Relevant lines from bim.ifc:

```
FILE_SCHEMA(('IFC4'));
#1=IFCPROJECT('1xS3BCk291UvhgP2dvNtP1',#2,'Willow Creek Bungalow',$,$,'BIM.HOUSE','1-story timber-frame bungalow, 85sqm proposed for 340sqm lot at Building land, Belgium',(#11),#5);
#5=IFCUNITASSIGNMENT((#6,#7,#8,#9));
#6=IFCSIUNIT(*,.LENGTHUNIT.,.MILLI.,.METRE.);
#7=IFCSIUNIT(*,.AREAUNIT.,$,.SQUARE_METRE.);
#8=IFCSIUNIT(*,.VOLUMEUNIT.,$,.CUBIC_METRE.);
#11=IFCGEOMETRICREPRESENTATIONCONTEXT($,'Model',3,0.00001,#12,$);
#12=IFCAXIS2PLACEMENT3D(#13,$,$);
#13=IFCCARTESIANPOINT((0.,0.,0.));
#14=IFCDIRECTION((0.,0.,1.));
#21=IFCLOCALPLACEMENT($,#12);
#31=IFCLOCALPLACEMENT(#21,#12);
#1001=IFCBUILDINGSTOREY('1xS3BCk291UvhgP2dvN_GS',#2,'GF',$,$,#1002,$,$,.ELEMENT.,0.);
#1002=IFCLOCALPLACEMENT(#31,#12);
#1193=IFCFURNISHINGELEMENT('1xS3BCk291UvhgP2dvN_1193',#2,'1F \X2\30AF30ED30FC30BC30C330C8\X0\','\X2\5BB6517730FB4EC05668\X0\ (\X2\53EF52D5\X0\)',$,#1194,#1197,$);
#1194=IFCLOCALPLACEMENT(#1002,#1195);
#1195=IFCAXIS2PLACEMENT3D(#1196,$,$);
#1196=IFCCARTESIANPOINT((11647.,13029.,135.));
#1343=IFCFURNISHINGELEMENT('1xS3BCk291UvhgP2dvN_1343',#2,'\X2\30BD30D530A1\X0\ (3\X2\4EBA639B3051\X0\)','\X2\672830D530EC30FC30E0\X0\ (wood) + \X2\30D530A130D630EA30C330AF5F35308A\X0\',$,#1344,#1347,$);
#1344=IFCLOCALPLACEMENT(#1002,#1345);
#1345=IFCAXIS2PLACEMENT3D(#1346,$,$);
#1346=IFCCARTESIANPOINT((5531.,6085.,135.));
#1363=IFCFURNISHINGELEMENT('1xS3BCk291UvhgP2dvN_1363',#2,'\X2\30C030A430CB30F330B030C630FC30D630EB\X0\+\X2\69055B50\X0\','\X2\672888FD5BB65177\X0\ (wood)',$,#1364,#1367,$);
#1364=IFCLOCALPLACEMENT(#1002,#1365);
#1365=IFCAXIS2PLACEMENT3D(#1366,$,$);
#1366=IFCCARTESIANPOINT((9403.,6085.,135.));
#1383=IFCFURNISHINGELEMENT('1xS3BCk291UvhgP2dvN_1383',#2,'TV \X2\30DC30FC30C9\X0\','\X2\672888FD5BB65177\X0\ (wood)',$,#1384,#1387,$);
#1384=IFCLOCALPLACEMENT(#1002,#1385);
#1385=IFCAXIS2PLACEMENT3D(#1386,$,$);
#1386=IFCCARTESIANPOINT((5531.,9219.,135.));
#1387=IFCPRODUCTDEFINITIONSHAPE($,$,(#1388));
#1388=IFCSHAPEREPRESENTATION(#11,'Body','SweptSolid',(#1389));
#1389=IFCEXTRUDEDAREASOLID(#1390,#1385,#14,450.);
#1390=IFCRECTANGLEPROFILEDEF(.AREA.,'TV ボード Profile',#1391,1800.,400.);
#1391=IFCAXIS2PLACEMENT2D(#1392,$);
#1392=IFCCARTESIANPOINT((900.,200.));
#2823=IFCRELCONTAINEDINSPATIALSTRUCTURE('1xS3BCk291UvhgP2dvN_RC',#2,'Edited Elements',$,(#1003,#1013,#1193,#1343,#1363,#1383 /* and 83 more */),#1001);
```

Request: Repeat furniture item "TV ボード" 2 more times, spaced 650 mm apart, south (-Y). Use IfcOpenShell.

```python
import numpy as np
import ifcopenshell
import ifcopenshell.api.geometry
import ifcopenshell.api.root
import ifcopenshell.util.element
import ifcopenshell.util.placement
import ifcopenshell.util.unit

model = ifcopenshell.open("bim.ifc")
unit_scale = ifcopenshell.util.unit.calculate_unit_scale(model)


def reuse_history(source, copy):
    """copy_class also copies each property set's owner history, people and application; keep the originals."""
    for rel in copy.IsDefinedBy:
        if rel.is_a("IfcRelDefinesByProperties") and (history := rel.RelatingPropertyDefinition.OwnerHistory):
            rel.RelatingPropertyDefinition.OwnerHistory = source.OwnerHistory
            ifcopenshell.util.element.remove_deep2(model, history)


source = model.by_id(1383)
base = ifcopenshell.util.placement.get_local_placement(source.ObjectPlacement)
step = np.array([0.0, -1.0, 0.0]) * 0.65 / unit_scale

for i in range(1, 3):
    copy = ifcopenshell.api.root.copy_class(model, product=source)
    copy.Representation = ifcopenshell.util.element.copy_deep(
        model, source.Representation, exclude=["IfcGeometricRepresentationContext", "IfcRepresentationMap"]
    )
    reuse_history(source, copy)
    matrix = base.copy()
    matrix[:3, 3] += i * step
    print("added at", matrix[:3, 3].round(3) + 0.0)
    ifcopenshell.api.geometry.edit_object_placement(model, product=copy, matrix=matrix, is_si=False)

model.write("bim_updated.ifc")
```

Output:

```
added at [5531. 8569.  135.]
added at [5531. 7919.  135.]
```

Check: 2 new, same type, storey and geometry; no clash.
